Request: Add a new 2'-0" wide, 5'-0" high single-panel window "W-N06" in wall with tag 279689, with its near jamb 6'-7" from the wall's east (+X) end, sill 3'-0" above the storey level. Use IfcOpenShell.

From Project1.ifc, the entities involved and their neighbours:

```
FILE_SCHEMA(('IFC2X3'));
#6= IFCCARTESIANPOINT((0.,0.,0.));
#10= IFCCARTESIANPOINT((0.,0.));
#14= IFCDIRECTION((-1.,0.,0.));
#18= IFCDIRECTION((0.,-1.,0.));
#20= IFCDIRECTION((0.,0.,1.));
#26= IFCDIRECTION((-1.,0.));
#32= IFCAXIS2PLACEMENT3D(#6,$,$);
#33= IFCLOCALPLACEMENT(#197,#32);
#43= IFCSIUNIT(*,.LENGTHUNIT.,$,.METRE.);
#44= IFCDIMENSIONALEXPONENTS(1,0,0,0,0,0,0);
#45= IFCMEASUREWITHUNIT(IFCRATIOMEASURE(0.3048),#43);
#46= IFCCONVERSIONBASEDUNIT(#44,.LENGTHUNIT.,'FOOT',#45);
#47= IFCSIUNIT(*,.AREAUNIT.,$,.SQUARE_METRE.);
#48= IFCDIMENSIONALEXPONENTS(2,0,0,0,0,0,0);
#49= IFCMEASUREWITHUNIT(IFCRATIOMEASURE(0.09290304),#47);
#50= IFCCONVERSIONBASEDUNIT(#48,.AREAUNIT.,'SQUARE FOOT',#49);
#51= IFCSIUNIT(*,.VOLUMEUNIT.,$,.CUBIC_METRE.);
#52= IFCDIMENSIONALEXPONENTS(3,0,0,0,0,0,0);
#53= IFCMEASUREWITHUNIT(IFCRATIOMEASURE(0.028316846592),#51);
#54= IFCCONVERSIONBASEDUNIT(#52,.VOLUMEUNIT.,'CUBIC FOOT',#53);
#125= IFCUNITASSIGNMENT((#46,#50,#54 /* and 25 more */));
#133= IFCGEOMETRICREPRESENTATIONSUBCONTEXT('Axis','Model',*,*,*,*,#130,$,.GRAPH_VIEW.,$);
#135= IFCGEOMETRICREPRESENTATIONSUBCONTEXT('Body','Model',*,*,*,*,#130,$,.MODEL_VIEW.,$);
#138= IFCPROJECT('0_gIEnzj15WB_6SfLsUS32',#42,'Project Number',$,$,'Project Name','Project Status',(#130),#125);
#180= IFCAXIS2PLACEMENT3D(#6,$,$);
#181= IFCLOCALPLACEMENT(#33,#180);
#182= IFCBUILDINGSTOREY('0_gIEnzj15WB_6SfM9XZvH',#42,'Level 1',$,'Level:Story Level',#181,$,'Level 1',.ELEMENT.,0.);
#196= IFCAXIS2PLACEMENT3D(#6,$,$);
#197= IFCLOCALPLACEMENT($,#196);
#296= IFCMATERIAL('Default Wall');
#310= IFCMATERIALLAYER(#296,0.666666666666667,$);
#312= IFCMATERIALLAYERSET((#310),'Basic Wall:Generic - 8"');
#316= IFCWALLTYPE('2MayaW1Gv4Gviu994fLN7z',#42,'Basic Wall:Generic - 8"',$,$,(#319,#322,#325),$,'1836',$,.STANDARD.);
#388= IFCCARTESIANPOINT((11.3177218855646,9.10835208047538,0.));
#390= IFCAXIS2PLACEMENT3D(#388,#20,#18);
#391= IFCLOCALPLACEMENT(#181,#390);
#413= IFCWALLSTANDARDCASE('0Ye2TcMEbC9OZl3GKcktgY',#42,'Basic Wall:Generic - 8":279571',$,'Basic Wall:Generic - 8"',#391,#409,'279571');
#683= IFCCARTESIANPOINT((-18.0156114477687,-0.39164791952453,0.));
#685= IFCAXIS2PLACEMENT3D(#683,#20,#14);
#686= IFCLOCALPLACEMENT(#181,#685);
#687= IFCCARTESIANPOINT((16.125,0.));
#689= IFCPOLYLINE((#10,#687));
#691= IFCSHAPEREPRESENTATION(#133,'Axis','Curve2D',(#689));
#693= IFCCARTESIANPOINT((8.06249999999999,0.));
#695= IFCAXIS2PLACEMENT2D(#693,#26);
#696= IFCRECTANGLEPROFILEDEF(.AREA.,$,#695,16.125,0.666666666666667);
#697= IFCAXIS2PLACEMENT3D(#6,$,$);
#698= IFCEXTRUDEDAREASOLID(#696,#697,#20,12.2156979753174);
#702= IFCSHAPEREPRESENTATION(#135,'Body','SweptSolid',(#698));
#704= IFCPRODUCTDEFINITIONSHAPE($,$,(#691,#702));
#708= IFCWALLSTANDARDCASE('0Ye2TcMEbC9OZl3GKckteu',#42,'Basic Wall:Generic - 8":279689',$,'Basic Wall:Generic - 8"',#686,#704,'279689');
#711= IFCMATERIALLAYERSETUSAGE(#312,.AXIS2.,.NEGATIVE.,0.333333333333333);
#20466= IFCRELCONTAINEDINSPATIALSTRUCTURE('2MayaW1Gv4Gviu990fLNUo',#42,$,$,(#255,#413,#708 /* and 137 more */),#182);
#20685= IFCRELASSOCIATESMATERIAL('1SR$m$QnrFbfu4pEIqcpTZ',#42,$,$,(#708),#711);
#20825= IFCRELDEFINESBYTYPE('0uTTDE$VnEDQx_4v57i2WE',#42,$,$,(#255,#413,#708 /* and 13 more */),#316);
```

```python
import numpy as np
import ifcopenshell
import ifcopenshell.api.feature
import ifcopenshell.api.geometry
import ifcopenshell.api.root
import ifcopenshell.api.spatial
import ifcopenshell.api.type
import ifcopenshell.geom
import ifcopenshell.util.element
import ifcopenshell.util.placement
import ifcopenshell.util.representation
import ifcopenshell.util.shape
import ifcopenshell.util.unit

model = ifcopenshell.open("Project1.ifc")
unit_scale = ifcopenshell.util.unit.calculate_unit_scale(model)
settings = ifcopenshell.geom.settings()


def volume(element):
    """Net volume in cubic metres, openings subtracted."""
    shape = ifcopenshell.geom.create_shape(settings, element)
    return ifcopenshell.util.shape.get_volume(shape.geometry)


wall = model.by_guid("0Ye2TcMEbC9OZl3GKckteu")
storey = ifcopenshell.util.element.get_container(wall, ifc_class="IfcBuildingStorey")
context = ifcopenshell.util.representation.get_context(model, "Model", "Body", "MODEL_VIEW")
before = volume(wall)

width, height, from_end, sill = 0.6096, 1.524, 2.0066, 0.9144  # metres

# The wall runs along its own X axis, and the end named is its -X end.
wall_shape = ifcopenshell.geom.create_shape(settings, wall)
x, y, z = ifcopenshell.util.shape.get_vertices(wall_shape.geometry).T
start = x.min() + from_end
face, thickness = float(y.min()), float(y.max() - y.min())
wall_matrix = ifcopenshell.util.placement.get_local_placement(wall.ObjectPlacement)
level = ifcopenshell.util.placement.get_local_placement(storey.ObjectPlacement)[2, 3]


def in_wall(x, y):
    """Placement at x, y metres in the wall's axes, at sill height."""
    matrix = wall_matrix.copy()
    matrix[:, 3] = wall_matrix @ np.array([x / unit_scale, y / unit_scale, 0.0, 1.0])
    matrix[2, 3] = level + sill / unit_scale
    return matrix


# Opening: a box that overshoots both wall faces by 50 mm.
opening = ifcopenshell.api.root.create_entity(model, ifc_class="IfcOpeningElement")
box = ifcopenshell.api.geometry.add_wall_representation(
    model, context=context, length=width, height=height, thickness=thickness + 0.1
)
ifcopenshell.api.geometry.assign_representation(model, product=opening, representation=box)
ifcopenshell.api.geometry.edit_object_placement(model, product=opening, matrix=in_wall(start, face - 0.05), is_si=False)
ifcopenshell.api.feature.add_feature(model, feature=opening, element=wall)

window = ifcopenshell.api.root.create_entity(model, ifc_class="IfcWindow", name="W-N06")
window.OverallWidth, window.OverallHeight = width / unit_scale, height / unit_scale
body = ifcopenshell.api.geometry.add_window_representation(
    model,
    context=context,
    overall_width=window.OverallWidth,
    overall_height=window.OverallHeight,
    partition_type="SINGLE_PANEL",
)
ifcopenshell.api.geometry.assign_representation(model, product=window, representation=body)
ifcopenshell.api.spatial.assign_container(model, products=[window], relating_structure=storey)
fills = ifcopenshell.api.feature.add_filling(model, opening=opening, element=window)
fills.OwnerHistory = window.OwnerHistory  # required in IFC2X3

# IFC2X3 keeps the operation on the window style.
style = ifcopenshell.api.root.create_entity(model, ifc_class="IfcWindowStyle", name="W-N06")
style.OperationType, style.ConstructionType = "SINGLE_PANEL", "NOTDEFINED"
style.ParameterTakesPrecedence = style.Sizeable = False
ifcopenshell.api.type.assign_type(model, related_objects=[window], relating_type=style)

# Centre the window in the wall's thickness.
ifcopenshell.api.geometry.edit_object_placement(model, product=window, matrix=in_wall(start, face), is_si=False)
window_shape = ifcopenshell.geom.create_shape(settings, window)
depth = ifcopenshell.util.shape.get_vertices(window_shape.geometry)[:, 1]
offset = face + thickness / 2 - (depth.min() + depth.max()) / 2
ifcopenshell.api.geometry.edit_object_placement(model, product=window, matrix=in_wall(start, offset), is_si=False)

after = volume(wall)

print(f"wall volume {before:.3f} -> {after:.3f} m3")

model.write("Project1_edited.ifc")
```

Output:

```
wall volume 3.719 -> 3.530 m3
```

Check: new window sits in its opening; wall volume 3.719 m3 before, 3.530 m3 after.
